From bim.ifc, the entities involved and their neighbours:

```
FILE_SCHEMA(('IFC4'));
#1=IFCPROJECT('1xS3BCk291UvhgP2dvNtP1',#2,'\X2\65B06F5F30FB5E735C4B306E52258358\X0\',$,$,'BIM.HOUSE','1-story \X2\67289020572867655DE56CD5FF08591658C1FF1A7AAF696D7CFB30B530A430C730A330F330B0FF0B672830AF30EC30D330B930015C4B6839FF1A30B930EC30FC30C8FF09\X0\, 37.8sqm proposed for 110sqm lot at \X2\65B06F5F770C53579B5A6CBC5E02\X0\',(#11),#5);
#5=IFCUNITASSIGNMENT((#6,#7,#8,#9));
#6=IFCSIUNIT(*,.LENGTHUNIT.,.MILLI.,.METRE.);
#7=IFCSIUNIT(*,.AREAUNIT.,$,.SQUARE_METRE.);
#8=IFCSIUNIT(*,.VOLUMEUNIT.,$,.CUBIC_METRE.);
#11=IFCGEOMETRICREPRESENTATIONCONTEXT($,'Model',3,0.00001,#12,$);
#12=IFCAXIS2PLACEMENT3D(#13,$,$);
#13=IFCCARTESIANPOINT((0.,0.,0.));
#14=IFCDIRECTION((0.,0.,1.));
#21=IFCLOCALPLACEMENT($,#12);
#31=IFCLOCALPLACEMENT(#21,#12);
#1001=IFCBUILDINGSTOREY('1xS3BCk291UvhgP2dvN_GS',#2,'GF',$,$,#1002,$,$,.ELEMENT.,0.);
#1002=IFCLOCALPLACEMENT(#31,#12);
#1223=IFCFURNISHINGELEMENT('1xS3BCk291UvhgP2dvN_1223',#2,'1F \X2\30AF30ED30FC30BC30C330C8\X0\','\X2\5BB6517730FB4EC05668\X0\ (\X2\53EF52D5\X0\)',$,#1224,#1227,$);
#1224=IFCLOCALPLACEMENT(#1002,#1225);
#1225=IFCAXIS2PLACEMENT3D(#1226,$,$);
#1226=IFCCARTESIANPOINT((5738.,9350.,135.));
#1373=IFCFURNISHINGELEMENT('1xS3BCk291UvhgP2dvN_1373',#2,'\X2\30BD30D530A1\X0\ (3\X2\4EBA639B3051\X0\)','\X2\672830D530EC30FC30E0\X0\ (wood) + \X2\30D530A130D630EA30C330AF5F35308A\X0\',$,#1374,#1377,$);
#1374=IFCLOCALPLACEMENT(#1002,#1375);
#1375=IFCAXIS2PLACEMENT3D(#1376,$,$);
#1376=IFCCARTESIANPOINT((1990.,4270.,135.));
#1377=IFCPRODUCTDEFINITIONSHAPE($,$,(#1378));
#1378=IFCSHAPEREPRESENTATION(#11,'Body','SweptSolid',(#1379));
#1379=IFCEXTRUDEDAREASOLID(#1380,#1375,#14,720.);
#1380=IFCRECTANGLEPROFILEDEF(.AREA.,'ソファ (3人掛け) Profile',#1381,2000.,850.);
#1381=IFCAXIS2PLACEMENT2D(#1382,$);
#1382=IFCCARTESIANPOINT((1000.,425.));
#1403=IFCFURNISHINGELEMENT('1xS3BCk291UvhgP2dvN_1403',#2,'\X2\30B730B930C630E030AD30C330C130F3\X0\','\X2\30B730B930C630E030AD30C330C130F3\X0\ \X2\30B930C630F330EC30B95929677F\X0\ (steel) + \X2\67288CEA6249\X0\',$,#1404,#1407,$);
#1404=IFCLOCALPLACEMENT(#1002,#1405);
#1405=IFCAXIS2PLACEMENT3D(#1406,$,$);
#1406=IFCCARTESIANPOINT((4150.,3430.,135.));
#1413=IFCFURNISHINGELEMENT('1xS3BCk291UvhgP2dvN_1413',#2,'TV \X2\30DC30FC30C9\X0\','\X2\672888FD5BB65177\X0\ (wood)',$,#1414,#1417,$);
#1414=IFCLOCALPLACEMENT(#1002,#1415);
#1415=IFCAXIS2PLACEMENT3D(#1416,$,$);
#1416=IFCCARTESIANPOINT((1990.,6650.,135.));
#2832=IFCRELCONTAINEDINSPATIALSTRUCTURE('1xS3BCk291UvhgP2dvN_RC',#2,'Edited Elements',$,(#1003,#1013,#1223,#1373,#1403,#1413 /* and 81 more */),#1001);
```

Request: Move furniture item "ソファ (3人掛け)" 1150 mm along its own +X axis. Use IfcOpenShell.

```python
import ifcopenshell
import ifcopenshell.api.geometry
import ifcopenshell.util.placement

model = ifcopenshell.open("bim.ifc")

item = model.by_guid("1xS3BCk291UvhgP2dvN_1373")
matrix = ifcopenshell.util.placement.get_local_placement(item.ObjectPlacement)
matrix[:3, 3] += matrix[:3, 0] * 1150.0
ifcopenshell.api.geometry.edit_object_placement(model, product=item, matrix=matrix, is_si=False)

print(ifcopenshell.util.placement.get_local_placement(item.ObjectPlacement).round(3) + 0.0)

model.write("bim_v2.ifc")
```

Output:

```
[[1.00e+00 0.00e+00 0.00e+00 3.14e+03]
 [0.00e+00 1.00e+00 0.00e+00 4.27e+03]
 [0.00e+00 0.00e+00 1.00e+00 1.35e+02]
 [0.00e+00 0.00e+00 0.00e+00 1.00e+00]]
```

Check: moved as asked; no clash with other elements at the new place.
